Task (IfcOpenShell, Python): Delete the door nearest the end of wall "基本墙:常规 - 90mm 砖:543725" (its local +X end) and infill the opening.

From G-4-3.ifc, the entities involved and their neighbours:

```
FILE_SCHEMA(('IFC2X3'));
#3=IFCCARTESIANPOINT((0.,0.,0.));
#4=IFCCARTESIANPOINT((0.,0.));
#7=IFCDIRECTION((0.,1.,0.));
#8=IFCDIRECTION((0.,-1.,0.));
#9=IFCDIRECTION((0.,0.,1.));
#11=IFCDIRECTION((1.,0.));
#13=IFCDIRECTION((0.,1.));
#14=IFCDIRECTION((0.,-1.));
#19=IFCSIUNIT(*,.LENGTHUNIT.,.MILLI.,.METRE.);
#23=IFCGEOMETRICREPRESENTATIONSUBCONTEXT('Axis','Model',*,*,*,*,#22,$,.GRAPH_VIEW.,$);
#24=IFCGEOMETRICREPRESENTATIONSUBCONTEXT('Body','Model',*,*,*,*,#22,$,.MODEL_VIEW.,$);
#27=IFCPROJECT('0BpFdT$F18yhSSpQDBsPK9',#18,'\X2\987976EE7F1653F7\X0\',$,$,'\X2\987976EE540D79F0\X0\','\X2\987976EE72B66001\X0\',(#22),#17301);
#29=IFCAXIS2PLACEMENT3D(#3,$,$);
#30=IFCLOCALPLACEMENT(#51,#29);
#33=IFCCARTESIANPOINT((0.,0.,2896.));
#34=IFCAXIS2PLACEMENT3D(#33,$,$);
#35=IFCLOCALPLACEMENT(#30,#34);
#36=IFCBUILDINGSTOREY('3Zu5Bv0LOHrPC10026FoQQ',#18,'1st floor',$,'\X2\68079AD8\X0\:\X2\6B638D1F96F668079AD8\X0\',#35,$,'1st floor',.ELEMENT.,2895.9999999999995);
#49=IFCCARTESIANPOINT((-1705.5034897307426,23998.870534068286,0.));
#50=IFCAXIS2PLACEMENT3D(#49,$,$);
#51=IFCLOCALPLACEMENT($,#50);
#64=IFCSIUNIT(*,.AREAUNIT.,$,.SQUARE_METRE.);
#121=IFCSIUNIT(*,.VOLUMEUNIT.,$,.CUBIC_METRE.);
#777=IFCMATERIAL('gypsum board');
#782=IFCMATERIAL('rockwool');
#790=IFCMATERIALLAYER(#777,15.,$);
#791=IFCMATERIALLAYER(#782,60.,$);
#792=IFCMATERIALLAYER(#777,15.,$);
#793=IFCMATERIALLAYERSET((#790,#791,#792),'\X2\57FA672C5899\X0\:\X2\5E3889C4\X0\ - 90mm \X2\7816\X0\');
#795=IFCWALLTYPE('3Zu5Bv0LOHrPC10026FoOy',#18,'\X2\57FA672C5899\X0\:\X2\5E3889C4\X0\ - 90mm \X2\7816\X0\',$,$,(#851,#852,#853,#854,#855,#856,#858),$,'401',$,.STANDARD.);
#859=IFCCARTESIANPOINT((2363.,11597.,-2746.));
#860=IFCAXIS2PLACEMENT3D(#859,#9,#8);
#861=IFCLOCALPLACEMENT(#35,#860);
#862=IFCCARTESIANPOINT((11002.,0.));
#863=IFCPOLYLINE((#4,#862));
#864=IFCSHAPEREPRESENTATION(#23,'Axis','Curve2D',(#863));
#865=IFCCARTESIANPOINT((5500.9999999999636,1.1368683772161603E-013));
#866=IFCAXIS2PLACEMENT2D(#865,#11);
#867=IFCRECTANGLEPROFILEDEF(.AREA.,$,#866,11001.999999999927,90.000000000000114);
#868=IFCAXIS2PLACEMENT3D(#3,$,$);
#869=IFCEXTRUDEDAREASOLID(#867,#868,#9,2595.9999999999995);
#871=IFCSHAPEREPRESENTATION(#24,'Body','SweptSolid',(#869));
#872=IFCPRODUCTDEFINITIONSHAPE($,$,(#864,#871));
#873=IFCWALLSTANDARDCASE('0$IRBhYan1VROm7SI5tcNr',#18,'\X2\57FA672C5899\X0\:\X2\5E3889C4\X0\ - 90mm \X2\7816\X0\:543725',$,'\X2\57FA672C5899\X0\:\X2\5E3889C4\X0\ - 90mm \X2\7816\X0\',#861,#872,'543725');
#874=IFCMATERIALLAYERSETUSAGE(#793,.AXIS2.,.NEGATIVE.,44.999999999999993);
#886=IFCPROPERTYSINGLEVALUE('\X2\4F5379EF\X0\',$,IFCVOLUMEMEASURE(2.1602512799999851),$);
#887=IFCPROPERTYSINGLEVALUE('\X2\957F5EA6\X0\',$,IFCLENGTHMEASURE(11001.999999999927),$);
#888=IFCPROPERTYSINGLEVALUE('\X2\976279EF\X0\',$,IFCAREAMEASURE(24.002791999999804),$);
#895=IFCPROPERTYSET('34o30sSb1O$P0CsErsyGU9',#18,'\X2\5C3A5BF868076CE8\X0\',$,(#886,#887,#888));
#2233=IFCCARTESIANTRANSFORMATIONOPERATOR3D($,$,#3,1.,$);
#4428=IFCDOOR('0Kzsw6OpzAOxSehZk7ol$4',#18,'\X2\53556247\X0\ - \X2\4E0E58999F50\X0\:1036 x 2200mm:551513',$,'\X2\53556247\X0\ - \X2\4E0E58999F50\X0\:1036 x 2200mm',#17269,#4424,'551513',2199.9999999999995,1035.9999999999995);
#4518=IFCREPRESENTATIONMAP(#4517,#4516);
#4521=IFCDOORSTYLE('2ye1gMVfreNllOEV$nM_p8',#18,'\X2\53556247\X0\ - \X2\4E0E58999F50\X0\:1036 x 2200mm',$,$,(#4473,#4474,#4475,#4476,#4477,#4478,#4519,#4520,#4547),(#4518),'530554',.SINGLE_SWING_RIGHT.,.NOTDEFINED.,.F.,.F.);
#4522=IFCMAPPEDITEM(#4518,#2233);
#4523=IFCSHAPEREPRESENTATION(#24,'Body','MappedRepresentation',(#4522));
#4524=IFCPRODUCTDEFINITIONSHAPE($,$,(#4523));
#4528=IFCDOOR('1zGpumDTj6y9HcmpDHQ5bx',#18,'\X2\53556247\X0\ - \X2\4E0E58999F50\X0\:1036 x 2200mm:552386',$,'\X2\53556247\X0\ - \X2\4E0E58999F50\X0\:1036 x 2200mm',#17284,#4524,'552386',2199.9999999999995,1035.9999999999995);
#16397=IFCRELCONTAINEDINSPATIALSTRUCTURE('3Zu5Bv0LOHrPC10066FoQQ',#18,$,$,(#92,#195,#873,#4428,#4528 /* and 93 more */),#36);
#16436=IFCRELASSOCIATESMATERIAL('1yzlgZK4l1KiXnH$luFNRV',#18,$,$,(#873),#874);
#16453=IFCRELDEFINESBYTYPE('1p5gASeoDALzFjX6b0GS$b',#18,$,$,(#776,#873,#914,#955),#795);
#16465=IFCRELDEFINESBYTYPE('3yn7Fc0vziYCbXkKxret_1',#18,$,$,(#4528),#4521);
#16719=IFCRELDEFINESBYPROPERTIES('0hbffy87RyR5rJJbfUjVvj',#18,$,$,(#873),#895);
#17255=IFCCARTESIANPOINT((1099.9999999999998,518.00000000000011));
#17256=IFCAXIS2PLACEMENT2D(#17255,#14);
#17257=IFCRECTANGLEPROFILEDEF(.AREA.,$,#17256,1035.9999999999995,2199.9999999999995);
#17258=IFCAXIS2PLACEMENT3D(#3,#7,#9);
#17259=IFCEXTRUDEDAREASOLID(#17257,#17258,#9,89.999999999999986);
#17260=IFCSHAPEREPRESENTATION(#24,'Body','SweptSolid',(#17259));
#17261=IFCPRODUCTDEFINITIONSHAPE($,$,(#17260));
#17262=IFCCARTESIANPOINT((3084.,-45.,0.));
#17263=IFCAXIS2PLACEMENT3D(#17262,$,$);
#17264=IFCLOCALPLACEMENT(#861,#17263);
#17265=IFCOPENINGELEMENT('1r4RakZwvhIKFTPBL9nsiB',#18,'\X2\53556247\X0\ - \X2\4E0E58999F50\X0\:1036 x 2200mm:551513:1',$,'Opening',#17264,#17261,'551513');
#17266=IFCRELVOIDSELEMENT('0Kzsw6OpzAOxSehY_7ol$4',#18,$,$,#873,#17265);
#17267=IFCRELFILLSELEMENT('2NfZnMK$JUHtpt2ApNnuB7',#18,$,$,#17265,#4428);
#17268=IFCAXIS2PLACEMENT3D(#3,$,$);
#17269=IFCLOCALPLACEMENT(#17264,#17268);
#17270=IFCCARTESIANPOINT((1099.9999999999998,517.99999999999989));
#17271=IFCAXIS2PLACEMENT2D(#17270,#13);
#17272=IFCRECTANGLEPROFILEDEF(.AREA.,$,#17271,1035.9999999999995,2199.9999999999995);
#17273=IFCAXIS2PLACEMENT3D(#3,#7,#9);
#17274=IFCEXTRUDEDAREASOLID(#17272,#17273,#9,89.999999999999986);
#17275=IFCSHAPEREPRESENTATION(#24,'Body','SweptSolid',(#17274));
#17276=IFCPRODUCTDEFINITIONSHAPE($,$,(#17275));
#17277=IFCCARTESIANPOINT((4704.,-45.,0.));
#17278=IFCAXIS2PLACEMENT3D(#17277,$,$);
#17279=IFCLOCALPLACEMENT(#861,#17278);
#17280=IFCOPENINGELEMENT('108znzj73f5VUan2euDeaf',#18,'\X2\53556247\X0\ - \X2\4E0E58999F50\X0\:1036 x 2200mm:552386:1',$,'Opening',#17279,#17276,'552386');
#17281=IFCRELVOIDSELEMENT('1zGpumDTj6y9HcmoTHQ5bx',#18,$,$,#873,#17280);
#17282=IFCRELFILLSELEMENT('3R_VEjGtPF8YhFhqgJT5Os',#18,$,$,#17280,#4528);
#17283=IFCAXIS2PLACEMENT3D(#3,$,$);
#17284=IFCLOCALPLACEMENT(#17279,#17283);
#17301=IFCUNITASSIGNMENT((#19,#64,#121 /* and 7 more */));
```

```python
import ifcopenshell
import ifcopenshell.api.feature
import ifcopenshell.api.pset
import ifcopenshell.api.root
import ifcopenshell.geom
import ifcopenshell.util.element
import ifcopenshell.util.shape
import ifcopenshell.util.unit

model = ifcopenshell.open("G-4-3.ifc")
area_scale = ifcopenshell.util.unit.calculate_unit_scale(model, "AREAUNIT")
volume_scale = ifcopenshell.util.unit.calculate_unit_scale(model, "VOLUMEUNIT")
settings = ifcopenshell.geom.settings()


def volume(element):
    """Net volume in cubic metres, openings subtracted."""
    shape = ifcopenshell.geom.create_shape(settings, element)
    return ifcopenshell.util.shape.get_volume(shape.geometry)


door = model.by_id(4528)
opening = door.FillsVoids[0].RelatingOpeningElement
wall = opening.VoidsElements[0].RelatingBuildingElement
before = volume(wall)

ifcopenshell.api.root.remove_product(model, product=door)
ifcopenshell.api.feature.remove_feature(model, feature=opening)

after = volume(wall)
thickness = 0.09  # wall thickness in metres

# Update the wall's stored quantities.
pset = model.by_id(ifcopenshell.util.element.get_pset(wall, "尺寸标注", should_inherit=False)["id"])
ifcopenshell.api.pset.edit_pset(model, pset=pset, properties={
    "体积": model.create_entity("IfcVolumeMeasure", after / volume_scale),
    "面积": model.create_entity("IfcAreaMeasure", after / thickness / area_scale),
})

print(f"wall volume {before:.3f} -> {after:.3f} m3")

model.write("G-4-3-out.ifc")
```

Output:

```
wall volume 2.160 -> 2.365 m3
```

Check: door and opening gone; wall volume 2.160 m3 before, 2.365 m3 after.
